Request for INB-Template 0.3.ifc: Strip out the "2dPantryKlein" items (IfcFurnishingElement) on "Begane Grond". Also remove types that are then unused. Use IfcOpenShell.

First a look at what the model holds.

```python
import ifcopenshell
import ifcopenshell.util.element

model = ifcopenshell.open("INB-Template 0.3.ifc")
print(model.schema)
storey = next(s for s in model.by_type("IfcBuildingStorey") if s.Name == "Begane Grond")
furniture = [e for e in ifcopenshell.util.element.get_decomposition(storey) if e.is_a("IfcFurnishingElement")]
seen = {}
for e in furniture:
    element_type = ifcopenshell.util.element.get_type(e)
    name = element_type.Name if element_type not in (None, e) else None
    seen[name] = seen.get(name, 0) + 1
for name, count in sorted(seen.items(), key=str):
    print(count, "x", name)
```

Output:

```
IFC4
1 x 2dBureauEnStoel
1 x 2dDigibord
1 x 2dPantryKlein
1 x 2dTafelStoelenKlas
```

```python
import ifcopenshell
import ifcopenshell.api.root
import ifcopenshell.util.element

model = ifcopenshell.open("INB-Template 0.3.ifc")

storey = next(s for s in model.by_type("IfcBuildingStorey") if s.Name == "Begane Grond")
furniture = [e for e in ifcopenshell.util.element.get_decomposition(storey) if e.is_a("IfcFurnishingElement")]
targets = [e for e in furniture if (t := ifcopenshell.util.element.get_type(e)) not in (None, e) and t.Name == "2dPantryKlein"]
types = {ifcopenshell.util.element.get_type(e) for e in targets} - {None, *targets}

for e in targets:
    ifcopenshell.api.root.remove_product(model, product=e)
print(len(targets), "removed")

unused = [t for t in types if not ifcopenshell.util.element.get_types(t)]
for t in unused:
    ifcopenshell.api.root.remove_product(model, product=t)
print(len(unused), "unused types removed")

model.write("INB-Template 0.3_rev.ifc")
```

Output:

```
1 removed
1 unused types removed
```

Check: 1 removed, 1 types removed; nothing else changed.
